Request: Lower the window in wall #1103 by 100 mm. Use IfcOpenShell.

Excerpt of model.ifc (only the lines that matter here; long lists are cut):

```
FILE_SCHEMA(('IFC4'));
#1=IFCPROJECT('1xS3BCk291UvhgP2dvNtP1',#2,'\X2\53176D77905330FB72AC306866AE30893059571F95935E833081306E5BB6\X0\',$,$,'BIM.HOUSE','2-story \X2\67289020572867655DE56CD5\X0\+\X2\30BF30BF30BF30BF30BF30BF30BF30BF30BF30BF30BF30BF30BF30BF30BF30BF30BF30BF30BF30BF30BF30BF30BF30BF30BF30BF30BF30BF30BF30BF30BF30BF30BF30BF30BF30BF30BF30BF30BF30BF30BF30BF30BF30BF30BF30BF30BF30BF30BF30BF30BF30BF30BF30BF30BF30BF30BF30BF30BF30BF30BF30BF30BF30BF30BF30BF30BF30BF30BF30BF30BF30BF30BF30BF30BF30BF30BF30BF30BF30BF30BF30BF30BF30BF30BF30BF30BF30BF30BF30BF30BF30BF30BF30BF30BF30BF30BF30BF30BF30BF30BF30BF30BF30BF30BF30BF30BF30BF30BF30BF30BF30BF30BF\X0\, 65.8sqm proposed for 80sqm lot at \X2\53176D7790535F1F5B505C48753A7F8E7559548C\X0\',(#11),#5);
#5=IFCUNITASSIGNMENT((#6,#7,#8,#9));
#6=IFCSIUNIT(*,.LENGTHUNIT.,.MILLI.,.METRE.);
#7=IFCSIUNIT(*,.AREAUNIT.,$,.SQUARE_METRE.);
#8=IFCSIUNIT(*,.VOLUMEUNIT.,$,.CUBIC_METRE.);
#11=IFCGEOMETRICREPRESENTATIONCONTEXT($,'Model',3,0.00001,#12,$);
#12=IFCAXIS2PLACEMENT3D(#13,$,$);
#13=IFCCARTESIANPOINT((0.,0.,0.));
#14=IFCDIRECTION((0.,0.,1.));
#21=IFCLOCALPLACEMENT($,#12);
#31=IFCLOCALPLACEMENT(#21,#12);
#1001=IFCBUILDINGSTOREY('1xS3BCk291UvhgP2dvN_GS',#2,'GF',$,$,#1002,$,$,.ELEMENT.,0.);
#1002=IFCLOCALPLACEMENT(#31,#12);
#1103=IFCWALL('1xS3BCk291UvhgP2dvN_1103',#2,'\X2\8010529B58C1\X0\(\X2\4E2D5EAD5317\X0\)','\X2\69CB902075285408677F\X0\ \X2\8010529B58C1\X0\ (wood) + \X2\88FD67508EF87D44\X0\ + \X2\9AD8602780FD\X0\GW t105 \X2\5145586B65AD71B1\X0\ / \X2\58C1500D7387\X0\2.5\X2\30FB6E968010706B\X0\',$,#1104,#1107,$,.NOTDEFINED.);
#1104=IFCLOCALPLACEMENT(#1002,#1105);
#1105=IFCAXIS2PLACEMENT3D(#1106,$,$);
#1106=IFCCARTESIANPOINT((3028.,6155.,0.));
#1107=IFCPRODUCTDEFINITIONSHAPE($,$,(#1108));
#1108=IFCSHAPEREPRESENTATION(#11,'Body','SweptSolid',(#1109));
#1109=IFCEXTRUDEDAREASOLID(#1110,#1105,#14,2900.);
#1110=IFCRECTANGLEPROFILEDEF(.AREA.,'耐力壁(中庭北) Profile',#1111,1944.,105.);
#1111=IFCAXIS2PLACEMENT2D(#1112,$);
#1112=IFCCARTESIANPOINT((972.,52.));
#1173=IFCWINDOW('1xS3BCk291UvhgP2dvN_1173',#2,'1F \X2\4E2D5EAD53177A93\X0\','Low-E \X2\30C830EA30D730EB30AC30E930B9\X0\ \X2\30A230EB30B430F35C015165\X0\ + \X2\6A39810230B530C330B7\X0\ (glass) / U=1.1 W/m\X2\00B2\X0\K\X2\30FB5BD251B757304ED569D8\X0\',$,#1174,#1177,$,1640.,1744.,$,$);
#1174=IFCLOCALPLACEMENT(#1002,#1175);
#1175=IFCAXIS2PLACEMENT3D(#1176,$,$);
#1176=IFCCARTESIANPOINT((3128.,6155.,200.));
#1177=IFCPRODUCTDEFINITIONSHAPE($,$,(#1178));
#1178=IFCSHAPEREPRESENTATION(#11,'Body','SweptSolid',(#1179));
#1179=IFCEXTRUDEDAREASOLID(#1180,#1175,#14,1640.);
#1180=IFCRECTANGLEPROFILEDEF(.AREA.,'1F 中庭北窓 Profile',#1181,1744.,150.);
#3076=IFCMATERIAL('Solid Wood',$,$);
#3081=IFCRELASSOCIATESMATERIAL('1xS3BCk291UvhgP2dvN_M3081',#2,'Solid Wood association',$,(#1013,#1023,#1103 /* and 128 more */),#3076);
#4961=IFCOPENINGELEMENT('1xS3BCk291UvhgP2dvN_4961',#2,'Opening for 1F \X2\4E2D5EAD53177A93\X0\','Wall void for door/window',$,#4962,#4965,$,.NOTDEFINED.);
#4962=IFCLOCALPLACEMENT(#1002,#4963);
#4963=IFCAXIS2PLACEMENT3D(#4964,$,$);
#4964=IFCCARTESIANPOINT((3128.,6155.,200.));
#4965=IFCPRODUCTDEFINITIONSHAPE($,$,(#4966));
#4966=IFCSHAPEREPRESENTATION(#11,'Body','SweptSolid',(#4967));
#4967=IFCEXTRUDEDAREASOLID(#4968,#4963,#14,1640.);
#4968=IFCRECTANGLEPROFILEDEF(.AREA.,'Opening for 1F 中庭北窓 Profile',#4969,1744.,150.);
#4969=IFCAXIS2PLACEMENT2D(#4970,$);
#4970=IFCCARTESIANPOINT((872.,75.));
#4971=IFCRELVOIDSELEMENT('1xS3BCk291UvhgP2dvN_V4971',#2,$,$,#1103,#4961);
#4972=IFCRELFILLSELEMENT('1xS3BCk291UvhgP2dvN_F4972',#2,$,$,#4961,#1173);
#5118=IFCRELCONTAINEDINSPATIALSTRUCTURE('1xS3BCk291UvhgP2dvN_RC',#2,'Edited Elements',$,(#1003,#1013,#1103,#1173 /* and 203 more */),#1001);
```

```python
import numpy as np
import ifcopenshell
import ifcopenshell.api.geometry
import ifcopenshell.util.placement
import ifcopenshell.util.unit

model = ifcopenshell.open("model.ifc")
unit_scale = ifcopenshell.util.unit.calculate_unit_scale(model)

window = model.by_id(1173)
opening = window.FillsVoids[0].RelatingOpeningElement
dz = -100.0

shift = np.array([0.0, 0.0, dz])
# The window is not placed relative to its opening, so move both.
for product in (opening, window):
    matrix = ifcopenshell.util.placement.get_local_placement(product.ObjectPlacement)
    matrix[:3, 3] += shift
    ifcopenshell.api.geometry.edit_object_placement(model, product=product, matrix=matrix, is_si=False)

print(f"moved by {dz * unit_scale:+.3f} m")

model.write("model_v2.ifc")
```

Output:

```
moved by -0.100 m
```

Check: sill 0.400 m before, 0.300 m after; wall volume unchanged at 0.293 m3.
